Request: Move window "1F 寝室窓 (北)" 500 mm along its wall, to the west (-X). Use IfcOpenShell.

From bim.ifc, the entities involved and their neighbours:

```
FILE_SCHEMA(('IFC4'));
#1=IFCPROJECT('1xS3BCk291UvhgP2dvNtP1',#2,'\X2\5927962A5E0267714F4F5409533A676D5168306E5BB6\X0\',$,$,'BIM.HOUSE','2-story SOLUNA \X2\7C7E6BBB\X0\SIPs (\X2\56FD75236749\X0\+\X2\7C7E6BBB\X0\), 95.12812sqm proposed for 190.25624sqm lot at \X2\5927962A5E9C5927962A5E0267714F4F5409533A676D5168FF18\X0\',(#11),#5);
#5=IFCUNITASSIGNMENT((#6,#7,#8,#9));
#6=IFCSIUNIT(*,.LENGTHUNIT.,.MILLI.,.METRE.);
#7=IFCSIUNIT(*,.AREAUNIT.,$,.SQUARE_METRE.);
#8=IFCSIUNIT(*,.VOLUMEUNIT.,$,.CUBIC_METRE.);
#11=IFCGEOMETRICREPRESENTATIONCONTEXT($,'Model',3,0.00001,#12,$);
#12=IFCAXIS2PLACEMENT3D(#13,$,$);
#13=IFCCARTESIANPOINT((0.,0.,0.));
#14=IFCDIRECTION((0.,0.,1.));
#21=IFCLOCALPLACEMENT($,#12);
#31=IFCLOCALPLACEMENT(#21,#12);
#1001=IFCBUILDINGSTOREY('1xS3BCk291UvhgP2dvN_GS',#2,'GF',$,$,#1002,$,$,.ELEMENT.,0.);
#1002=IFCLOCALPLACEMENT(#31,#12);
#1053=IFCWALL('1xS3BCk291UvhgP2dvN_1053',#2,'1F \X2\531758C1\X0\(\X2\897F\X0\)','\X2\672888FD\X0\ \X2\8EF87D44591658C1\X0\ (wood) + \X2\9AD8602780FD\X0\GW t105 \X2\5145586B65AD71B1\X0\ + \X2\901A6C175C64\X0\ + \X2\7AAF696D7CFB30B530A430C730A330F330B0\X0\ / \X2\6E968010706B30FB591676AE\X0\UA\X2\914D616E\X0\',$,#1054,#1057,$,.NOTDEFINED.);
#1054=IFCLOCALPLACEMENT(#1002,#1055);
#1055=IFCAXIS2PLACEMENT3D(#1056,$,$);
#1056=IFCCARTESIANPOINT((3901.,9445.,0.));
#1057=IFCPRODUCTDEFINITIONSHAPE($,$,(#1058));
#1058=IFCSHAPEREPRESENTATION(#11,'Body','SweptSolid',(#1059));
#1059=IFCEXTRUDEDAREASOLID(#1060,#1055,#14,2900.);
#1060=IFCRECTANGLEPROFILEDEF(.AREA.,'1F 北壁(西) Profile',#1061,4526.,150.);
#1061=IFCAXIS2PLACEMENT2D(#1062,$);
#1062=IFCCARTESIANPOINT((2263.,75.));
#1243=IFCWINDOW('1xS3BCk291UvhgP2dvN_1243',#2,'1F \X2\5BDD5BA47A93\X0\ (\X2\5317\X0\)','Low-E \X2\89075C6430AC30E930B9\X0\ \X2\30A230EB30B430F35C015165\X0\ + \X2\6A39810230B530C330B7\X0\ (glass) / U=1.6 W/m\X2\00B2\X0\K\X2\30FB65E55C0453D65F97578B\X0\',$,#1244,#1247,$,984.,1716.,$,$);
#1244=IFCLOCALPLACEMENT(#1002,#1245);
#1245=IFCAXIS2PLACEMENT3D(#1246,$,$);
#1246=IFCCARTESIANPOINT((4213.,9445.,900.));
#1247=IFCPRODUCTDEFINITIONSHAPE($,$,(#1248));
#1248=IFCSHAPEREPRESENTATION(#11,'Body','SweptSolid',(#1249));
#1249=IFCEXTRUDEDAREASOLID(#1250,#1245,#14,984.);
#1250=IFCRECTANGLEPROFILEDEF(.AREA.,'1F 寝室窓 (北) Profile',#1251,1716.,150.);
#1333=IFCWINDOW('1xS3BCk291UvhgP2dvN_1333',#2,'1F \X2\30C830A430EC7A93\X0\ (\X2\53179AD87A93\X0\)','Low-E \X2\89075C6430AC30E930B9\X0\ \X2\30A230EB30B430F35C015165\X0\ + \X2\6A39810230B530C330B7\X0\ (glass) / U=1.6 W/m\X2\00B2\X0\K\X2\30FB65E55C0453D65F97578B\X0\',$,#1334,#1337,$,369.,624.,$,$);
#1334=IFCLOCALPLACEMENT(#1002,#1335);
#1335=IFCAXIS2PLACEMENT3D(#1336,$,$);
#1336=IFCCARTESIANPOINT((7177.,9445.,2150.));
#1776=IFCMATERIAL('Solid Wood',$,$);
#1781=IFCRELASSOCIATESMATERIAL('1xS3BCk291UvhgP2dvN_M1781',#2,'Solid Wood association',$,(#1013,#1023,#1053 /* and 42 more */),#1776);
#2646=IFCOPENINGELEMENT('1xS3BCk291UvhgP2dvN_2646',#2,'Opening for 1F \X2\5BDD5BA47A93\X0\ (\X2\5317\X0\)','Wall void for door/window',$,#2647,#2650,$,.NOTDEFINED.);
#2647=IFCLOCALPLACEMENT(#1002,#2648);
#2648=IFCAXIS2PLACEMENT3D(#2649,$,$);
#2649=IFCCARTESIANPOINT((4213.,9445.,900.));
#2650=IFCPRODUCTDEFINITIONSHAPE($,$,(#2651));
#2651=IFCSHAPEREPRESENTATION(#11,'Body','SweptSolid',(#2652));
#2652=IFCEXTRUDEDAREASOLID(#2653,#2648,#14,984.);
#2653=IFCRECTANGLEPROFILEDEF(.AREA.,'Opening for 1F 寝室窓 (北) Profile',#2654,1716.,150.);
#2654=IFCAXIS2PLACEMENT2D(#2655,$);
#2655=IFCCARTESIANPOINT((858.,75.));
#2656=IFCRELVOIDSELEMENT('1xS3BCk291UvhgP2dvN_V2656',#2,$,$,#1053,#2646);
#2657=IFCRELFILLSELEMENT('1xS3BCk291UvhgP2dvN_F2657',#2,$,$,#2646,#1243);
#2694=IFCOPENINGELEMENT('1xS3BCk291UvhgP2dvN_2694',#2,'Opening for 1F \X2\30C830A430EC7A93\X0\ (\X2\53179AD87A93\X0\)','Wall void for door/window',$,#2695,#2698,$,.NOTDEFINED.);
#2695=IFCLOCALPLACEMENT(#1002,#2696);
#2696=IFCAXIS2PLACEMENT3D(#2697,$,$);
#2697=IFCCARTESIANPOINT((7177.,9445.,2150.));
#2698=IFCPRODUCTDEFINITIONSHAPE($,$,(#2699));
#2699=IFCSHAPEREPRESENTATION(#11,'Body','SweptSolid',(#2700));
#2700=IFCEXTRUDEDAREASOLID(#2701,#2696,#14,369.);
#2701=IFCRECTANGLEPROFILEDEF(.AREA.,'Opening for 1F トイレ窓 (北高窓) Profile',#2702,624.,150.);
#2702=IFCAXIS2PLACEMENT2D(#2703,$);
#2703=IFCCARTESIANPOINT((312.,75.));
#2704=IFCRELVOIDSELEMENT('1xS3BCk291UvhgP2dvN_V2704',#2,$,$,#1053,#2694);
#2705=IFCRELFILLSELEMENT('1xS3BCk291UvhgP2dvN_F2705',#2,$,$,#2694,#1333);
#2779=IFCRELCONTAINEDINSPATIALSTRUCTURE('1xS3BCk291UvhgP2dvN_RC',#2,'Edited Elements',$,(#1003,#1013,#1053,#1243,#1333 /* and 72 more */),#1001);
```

```python
import ifcopenshell
import ifcopenshell.api.geometry
import ifcopenshell.util.placement
import ifcopenshell.util.unit

model = ifcopenshell.open("bim.ifc")
unit_scale = ifcopenshell.util.unit.calculate_unit_scale(model)

window = model.by_id(1243)
opening = window.FillsVoids[0].RelatingOpeningElement
wall = opening.VoidsElements[0].RelatingBuildingElement

wall_matrix = ifcopenshell.util.placement.get_local_placement(wall.ObjectPlacement)
shift = wall_matrix[:3, 0] * -0.5 / unit_scale
before = ifcopenshell.util.placement.get_local_placement(window.ObjectPlacement)[:3, 3].copy()

# The window is not placed relative to its opening, so move both.
for product in (opening, window):
    matrix = ifcopenshell.util.placement.get_local_placement(product.ObjectPlacement)
    matrix[:3, 3] += shift
    ifcopenshell.api.geometry.edit_object_placement(model, product=product, matrix=matrix, is_si=False)

after = ifcopenshell.util.placement.get_local_placement(window.ObjectPlacement)[:3, 3]
print("window moved by", (after - before).round(3) + 0.0)

model.write("bim_edited.ifc")
```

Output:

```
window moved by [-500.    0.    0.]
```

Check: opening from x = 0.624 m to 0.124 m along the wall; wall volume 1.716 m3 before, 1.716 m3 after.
